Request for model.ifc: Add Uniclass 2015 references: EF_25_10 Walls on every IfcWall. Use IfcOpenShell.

First a look at what the model holds.

```python
import ifcopenshell

model = ifcopenshell.open("model.ifc")
print(model.schema)
print("classifications:", [c.Name for c in model.by_type("IfcClassification")])
for ifc_class in ("IfcDoor", "IfcRoof", "IfcStair", "IfcWall", "IfcWindow"):
    print(ifc_class, len(model.by_type(ifc_class)))
```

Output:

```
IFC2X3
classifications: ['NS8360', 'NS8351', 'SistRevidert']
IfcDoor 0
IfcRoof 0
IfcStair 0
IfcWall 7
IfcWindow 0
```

```python
import ifcopenshell
import ifcopenshell.api.classification

model = ifcopenshell.open("model.ifc")

# IFC2X3 requires Source and Edition and has no link from the project to the system.
system = model.create_entity("IfcClassification", Source="NBS", Edition="2015", Name="Uniclass 2015")

codes = {
    "IfcWall": ("EF_25_10", "Walls"),
}
for ifc_class, (code, name) in codes.items():
    products = model.by_type(ifc_class)
    ifcopenshell.api.classification.add_reference(
        model, products=products, classification=system, identification=code, name=name
    )
    print(code, len(products))

model.write("model-out.ifc")
```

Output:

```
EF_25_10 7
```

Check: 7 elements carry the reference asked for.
